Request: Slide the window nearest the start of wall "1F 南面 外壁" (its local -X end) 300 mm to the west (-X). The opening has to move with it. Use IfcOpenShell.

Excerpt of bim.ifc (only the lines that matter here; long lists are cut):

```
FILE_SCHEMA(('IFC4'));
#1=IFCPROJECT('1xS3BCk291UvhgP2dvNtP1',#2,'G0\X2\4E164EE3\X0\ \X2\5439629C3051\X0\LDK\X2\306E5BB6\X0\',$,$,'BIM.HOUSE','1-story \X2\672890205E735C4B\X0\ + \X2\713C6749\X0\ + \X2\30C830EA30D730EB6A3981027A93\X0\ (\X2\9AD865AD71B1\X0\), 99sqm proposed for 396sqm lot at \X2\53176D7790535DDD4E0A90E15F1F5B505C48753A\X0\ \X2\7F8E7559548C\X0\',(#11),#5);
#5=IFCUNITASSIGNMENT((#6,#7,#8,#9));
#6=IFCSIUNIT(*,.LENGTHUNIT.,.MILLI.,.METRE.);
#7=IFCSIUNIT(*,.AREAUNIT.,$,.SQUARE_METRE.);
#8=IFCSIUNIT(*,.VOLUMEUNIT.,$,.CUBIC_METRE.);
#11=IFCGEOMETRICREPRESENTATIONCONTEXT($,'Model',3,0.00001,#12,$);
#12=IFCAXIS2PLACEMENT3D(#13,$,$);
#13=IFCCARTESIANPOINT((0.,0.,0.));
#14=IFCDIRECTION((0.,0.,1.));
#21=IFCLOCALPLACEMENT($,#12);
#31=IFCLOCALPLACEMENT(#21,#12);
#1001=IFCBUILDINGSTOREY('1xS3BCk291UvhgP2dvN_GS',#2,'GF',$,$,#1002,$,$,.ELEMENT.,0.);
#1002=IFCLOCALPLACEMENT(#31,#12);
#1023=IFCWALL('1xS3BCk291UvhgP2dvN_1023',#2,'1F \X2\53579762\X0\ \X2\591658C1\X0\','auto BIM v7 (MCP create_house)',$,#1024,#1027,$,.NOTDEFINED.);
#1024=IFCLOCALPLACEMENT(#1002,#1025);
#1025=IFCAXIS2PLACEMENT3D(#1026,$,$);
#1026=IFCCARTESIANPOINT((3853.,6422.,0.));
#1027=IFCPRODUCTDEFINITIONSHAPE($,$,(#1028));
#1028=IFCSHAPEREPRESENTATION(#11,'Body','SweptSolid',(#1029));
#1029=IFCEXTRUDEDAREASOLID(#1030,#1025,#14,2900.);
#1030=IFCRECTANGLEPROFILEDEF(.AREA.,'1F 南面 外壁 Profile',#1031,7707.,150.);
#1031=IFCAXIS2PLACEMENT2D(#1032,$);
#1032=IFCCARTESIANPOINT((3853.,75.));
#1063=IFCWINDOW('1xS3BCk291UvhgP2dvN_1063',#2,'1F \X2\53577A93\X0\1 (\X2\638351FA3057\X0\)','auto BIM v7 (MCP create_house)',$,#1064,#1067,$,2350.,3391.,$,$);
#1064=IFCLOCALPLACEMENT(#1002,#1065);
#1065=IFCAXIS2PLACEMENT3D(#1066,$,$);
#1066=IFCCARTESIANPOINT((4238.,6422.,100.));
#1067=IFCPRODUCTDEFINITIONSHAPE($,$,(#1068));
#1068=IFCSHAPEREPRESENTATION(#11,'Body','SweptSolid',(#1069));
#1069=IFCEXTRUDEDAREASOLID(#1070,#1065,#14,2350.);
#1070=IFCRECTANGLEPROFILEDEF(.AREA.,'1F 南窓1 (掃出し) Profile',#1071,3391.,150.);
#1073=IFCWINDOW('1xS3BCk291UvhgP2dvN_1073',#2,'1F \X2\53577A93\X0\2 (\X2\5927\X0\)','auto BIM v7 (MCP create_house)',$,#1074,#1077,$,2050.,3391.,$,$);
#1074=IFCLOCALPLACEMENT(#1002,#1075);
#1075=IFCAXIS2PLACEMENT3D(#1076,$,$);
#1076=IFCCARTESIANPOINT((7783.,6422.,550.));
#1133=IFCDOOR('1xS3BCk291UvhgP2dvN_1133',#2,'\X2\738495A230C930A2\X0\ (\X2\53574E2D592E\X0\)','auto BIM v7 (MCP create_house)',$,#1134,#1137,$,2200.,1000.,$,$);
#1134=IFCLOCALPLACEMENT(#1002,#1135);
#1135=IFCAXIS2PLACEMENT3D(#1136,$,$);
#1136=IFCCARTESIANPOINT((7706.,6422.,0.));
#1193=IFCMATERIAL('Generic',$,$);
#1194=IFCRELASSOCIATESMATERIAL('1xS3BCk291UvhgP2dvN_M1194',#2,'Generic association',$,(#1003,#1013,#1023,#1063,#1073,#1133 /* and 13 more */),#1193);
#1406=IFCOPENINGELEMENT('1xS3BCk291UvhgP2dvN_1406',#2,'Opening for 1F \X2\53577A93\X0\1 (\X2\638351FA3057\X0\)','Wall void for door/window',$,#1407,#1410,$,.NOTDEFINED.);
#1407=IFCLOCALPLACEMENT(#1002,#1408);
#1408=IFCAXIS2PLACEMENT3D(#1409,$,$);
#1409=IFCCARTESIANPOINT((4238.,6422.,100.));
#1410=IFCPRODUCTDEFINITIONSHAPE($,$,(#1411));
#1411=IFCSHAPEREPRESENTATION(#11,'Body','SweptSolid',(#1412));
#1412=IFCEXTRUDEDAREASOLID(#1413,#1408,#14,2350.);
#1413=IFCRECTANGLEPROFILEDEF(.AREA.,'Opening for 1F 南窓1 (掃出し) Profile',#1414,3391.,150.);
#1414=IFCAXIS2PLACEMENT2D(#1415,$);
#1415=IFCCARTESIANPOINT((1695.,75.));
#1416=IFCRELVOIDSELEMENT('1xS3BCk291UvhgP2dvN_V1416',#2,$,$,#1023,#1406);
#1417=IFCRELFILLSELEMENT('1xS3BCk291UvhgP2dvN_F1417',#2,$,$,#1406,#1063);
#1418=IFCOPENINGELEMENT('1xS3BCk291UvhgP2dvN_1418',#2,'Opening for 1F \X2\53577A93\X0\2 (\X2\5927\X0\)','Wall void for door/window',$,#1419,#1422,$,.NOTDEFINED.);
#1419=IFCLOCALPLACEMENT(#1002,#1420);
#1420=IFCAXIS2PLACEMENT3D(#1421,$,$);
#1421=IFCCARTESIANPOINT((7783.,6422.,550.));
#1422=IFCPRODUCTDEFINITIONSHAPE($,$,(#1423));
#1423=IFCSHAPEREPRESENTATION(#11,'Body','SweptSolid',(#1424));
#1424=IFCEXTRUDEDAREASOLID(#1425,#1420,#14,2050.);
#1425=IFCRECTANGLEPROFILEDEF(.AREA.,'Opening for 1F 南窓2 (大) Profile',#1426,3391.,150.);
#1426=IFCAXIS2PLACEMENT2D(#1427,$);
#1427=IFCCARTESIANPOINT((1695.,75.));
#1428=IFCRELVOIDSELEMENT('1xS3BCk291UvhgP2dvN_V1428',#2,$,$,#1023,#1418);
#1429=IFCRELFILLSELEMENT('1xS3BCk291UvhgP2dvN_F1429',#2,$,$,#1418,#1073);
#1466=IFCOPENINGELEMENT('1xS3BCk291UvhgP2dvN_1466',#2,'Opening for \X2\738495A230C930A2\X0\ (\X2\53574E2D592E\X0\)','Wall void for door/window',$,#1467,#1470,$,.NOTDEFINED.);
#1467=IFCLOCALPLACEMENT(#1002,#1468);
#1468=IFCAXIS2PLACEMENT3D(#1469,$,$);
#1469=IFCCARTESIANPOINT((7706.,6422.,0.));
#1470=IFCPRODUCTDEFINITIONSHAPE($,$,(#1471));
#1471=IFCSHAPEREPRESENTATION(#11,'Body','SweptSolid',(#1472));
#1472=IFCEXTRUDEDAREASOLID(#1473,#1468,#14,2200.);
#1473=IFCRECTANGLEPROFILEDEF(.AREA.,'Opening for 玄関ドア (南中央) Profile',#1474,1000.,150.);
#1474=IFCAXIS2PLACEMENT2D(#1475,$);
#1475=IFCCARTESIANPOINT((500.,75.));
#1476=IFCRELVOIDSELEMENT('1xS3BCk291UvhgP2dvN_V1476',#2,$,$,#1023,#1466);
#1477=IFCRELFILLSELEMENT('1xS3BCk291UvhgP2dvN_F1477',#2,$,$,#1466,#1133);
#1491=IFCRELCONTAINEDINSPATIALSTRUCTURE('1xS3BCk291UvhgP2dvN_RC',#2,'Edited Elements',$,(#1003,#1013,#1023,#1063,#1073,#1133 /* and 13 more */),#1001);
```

```python
import ifcopenshell
import ifcopenshell.api.geometry
import ifcopenshell.util.placement
import ifcopenshell.util.unit

model = ifcopenshell.open("bim.ifc")
unit_scale = ifcopenshell.util.unit.calculate_unit_scale(model)

window = model.by_id(1063)
opening = window.FillsVoids[0].RelatingOpeningElement
wall = opening.VoidsElements[0].RelatingBuildingElement

wall_matrix = ifcopenshell.util.placement.get_local_placement(wall.ObjectPlacement)
shift = wall_matrix[:3, 0] * -0.3 / unit_scale
before = ifcopenshell.util.placement.get_local_placement(window.ObjectPlacement)[:3, 3].copy()

# The window is not placed relative to its opening, so move both.
for product in (opening, window):
    matrix = ifcopenshell.util.placement.get_local_placement(product.ObjectPlacement)
    matrix[:3, 3] += shift
    ifcopenshell.api.geometry.edit_object_placement(model, product=product, matrix=matrix, is_si=False)

after = ifcopenshell.util.placement.get_local_placement(window.ObjectPlacement)[:3, 3]
print("window moved by", (after - before).round(3) + 0.0)

model.write("bim_v2.ifc")
```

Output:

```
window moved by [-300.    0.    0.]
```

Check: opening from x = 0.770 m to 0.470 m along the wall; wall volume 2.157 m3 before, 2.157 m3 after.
